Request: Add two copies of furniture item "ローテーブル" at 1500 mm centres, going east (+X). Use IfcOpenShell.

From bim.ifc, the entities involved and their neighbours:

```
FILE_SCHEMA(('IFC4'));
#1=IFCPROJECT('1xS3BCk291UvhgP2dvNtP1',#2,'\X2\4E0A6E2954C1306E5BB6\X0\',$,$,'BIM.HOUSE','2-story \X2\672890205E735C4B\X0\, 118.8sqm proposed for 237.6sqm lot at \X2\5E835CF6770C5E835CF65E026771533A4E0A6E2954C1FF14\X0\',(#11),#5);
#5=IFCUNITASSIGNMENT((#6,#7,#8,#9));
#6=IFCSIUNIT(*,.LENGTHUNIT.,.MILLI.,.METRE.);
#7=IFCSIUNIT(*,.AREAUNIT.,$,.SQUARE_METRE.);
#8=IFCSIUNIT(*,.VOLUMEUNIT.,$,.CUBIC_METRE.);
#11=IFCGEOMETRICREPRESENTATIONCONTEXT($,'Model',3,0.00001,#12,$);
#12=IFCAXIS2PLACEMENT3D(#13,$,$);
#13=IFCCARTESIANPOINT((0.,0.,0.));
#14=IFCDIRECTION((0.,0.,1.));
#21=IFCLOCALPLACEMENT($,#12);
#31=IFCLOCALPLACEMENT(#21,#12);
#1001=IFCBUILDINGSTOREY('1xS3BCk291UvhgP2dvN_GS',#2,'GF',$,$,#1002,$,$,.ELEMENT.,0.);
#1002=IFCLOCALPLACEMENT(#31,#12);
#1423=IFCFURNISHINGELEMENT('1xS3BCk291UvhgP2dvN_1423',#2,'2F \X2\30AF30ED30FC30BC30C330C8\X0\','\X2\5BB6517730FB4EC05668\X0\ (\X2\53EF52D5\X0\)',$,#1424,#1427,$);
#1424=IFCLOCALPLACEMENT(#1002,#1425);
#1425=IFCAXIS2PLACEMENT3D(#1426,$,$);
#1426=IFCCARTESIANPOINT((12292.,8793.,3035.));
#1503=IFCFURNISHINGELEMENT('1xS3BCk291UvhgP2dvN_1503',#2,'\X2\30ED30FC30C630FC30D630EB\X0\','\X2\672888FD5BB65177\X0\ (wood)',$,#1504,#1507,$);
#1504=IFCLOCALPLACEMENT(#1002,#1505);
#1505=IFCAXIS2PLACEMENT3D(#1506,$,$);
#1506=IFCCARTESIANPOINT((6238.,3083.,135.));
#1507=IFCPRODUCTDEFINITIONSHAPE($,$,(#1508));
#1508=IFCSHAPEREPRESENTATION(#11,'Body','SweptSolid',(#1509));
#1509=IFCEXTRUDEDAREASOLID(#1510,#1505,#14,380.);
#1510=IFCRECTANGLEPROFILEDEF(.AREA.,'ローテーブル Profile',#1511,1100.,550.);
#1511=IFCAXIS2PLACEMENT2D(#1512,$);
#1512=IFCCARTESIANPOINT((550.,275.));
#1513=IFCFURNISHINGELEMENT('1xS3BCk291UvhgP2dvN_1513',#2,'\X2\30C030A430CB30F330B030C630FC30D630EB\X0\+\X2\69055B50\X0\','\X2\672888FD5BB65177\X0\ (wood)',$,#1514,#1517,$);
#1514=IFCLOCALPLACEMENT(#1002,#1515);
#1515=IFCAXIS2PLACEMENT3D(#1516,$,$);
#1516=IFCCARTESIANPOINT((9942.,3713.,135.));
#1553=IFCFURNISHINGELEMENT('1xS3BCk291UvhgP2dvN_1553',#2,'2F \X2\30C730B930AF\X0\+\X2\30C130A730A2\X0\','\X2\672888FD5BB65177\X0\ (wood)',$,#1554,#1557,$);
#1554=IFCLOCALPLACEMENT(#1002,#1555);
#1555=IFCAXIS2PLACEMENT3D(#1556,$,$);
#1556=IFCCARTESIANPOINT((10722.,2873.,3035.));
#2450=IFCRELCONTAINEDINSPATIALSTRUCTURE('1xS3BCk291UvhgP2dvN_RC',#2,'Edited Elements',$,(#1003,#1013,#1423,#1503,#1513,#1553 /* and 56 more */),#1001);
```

```python
import numpy as np
import ifcopenshell
import ifcopenshell.api.geometry
import ifcopenshell.api.root
import ifcopenshell.util.element
import ifcopenshell.util.placement
import ifcopenshell.util.unit

model = ifcopenshell.open("bim.ifc")
unit_scale = ifcopenshell.util.unit.calculate_unit_scale(model)


def reuse_history(source, copy):
    """copy_class also copies each property set's owner history, people and application; keep the originals."""
    for rel in copy.IsDefinedBy:
        if rel.is_a("IfcRelDefinesByProperties") and (history := rel.RelatingPropertyDefinition.OwnerHistory):
            rel.RelatingPropertyDefinition.OwnerHistory = source.OwnerHistory
            ifcopenshell.util.element.remove_deep2(model, history)


source = model.by_guid("1xS3BCk291UvhgP2dvN_1503")
base = ifcopenshell.util.placement.get_local_placement(source.ObjectPlacement)
step = np.array([1.0, 0.0, 0.0]) * 1.5 / unit_scale

for i in range(1, 3):
    copy = ifcopenshell.api.root.copy_class(model, product=source)
    copy.Representation = ifcopenshell.util.element.copy_deep(
        model, source.Representation, exclude=["IfcGeometricRepresentationContext", "IfcRepresentationMap"]
    )
    reuse_history(source, copy)
    matrix = base.copy()
    matrix[:3, 3] += i * step
    print("added at", matrix[:3, 3].round(3) + 0.0)
    ifcopenshell.api.geometry.edit_object_placement(model, product=copy, matrix=matrix, is_si=False)

model.write("bim-out.ifc")
```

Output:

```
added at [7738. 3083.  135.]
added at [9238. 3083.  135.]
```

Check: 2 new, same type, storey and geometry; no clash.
